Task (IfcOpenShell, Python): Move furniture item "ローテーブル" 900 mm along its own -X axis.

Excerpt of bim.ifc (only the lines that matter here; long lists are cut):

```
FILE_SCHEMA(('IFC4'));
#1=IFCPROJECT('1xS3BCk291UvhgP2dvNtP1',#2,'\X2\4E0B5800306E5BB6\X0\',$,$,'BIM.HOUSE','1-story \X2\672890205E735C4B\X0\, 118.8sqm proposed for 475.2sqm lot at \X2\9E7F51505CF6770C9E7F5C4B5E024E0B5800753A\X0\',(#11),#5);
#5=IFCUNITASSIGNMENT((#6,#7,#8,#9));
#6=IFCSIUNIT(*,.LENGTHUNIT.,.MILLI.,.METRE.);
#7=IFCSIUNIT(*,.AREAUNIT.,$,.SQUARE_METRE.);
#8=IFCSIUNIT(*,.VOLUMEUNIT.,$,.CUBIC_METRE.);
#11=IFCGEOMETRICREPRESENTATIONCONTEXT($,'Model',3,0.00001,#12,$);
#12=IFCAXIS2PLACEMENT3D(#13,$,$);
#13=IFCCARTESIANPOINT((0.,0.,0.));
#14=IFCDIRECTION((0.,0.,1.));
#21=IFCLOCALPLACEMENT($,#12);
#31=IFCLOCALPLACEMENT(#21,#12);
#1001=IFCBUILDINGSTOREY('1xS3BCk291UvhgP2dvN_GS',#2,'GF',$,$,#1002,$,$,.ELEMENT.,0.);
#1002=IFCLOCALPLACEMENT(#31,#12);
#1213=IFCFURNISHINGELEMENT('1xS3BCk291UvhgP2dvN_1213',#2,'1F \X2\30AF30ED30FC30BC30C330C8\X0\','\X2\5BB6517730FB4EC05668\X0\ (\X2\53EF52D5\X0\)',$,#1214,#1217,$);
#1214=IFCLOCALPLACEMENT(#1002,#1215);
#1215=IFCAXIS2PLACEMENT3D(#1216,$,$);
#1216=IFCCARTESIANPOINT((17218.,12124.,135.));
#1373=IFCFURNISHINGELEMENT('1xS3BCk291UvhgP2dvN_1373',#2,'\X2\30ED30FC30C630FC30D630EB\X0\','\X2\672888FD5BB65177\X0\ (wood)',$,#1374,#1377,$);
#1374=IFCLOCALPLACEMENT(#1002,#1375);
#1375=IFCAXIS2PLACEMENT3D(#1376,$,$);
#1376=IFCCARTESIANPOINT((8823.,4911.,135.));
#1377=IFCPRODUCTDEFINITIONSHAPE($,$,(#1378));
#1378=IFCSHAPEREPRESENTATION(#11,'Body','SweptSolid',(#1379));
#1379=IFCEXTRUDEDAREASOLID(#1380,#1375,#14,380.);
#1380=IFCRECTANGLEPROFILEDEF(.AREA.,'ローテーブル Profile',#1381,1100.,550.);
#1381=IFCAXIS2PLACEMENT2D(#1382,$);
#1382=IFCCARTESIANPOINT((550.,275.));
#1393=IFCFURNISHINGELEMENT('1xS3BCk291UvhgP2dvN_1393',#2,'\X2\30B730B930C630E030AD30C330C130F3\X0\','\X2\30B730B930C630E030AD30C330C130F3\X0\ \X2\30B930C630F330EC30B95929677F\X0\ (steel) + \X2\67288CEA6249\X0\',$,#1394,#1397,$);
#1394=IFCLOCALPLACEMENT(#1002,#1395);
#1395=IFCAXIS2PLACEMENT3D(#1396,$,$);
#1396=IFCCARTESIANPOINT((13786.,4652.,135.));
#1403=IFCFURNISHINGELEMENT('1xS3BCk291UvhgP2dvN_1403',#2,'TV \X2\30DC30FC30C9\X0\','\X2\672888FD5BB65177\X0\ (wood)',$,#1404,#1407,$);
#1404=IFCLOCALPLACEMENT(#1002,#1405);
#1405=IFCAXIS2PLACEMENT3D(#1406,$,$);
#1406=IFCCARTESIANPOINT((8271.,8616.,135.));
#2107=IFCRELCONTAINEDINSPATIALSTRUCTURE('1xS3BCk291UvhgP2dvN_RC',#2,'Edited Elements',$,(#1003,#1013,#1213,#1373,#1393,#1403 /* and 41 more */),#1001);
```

```python
import ifcopenshell
import ifcopenshell.api.geometry
import ifcopenshell.util.placement

model = ifcopenshell.open("bim.ifc")

item = model.by_id(1373)
matrix = ifcopenshell.util.placement.get_local_placement(item.ObjectPlacement)
matrix[:3, 3] -= matrix[:3, 0] * 900.0
ifcopenshell.api.geometry.edit_object_placement(model, product=item, matrix=matrix, is_si=False)

print(ifcopenshell.util.placement.get_local_placement(item.ObjectPlacement).round(3) + 0.0)

model.write("bim_updated.ifc")
```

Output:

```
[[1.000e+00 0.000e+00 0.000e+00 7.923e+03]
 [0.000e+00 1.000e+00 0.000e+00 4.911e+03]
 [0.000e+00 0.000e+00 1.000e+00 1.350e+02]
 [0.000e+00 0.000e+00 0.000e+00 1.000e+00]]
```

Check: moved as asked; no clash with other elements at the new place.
